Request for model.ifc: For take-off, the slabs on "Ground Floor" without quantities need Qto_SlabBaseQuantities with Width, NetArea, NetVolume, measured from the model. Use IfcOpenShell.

First a look at what the model holds.

```python
import ifcopenshell
import ifcopenshell.util.element
import ifcopenshell.util.unit

model = ifcopenshell.open("model.ifc")
print(model.schema)
for unit_type in ("LENGTHUNIT", "AREAUNIT", "VOLUMEUNIT"):
    print(unit_type, ifcopenshell.util.unit.calculate_unit_scale(model, unit_type))
storey = next(s for s in model.by_type("IfcBuildingStorey") if s.Name == "Ground Floor")
slabs = [e for e in ifcopenshell.util.element.get_decomposition(storey) if e.is_a("IfcSlab")]
for e in sorted(slabs, key=lambda e: e.id()):
    print(e.id(), e.is_a(), e.Name, list(ifcopenshell.util.element.get_psets(e, qtos_only=True)), sep=" | ")
```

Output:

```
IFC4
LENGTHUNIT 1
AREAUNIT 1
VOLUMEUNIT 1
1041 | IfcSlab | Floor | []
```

```python
import ifcopenshell
import ifcopenshell.api.pset
import ifcopenshell.geom
import ifcopenshell.util.element
import ifcopenshell.util.shape
import ifcopenshell.util.unit

model = ifcopenshell.open("model.ifc")
unit_scale = ifcopenshell.util.unit.calculate_unit_scale(model)
area_scale = ifcopenshell.util.unit.calculate_unit_scale(model, "AREAUNIT")
volume_scale = ifcopenshell.util.unit.calculate_unit_scale(model, "VOLUMEUNIT")
settings = ifcopenshell.geom.settings()

storey = next(s for s in model.by_type("IfcBuildingStorey") if s.Name == "Ground Floor")
slabs = [e for e in ifcopenshell.util.element.get_decomposition(storey) if e.is_a("IfcSlab")]

for e in sorted(slabs, key=lambda e: e.id()):
    if ifcopenshell.util.element.get_psets(e, qtos_only=True, should_inherit=False):
        continue
    # Geometry comes back in metres, in the element's own axes.
    shape = ifcopenshell.geom.create_shape(settings, e)
    values = {
        "Width": ifcopenshell.util.shape.get_z(shape.geometry) / unit_scale,
        "NetArea": ifcopenshell.util.shape.get_footprint_area(shape.geometry) / area_scale,
        "NetVolume": ifcopenshell.util.shape.get_volume(shape.geometry) / volume_scale,
    }
    qto = ifcopenshell.api.pset.add_qto(model, product=e, name="Qto_SlabBaseQuantities")
    ifcopenshell.api.pset.edit_qto(model, qto=qto, properties=values)
    print(e.id(), {k: round(v, 3) for k, v in values.items()})

model.write("model_edited.ifc")
```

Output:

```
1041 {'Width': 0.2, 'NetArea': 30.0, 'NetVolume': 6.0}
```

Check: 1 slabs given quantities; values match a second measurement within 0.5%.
